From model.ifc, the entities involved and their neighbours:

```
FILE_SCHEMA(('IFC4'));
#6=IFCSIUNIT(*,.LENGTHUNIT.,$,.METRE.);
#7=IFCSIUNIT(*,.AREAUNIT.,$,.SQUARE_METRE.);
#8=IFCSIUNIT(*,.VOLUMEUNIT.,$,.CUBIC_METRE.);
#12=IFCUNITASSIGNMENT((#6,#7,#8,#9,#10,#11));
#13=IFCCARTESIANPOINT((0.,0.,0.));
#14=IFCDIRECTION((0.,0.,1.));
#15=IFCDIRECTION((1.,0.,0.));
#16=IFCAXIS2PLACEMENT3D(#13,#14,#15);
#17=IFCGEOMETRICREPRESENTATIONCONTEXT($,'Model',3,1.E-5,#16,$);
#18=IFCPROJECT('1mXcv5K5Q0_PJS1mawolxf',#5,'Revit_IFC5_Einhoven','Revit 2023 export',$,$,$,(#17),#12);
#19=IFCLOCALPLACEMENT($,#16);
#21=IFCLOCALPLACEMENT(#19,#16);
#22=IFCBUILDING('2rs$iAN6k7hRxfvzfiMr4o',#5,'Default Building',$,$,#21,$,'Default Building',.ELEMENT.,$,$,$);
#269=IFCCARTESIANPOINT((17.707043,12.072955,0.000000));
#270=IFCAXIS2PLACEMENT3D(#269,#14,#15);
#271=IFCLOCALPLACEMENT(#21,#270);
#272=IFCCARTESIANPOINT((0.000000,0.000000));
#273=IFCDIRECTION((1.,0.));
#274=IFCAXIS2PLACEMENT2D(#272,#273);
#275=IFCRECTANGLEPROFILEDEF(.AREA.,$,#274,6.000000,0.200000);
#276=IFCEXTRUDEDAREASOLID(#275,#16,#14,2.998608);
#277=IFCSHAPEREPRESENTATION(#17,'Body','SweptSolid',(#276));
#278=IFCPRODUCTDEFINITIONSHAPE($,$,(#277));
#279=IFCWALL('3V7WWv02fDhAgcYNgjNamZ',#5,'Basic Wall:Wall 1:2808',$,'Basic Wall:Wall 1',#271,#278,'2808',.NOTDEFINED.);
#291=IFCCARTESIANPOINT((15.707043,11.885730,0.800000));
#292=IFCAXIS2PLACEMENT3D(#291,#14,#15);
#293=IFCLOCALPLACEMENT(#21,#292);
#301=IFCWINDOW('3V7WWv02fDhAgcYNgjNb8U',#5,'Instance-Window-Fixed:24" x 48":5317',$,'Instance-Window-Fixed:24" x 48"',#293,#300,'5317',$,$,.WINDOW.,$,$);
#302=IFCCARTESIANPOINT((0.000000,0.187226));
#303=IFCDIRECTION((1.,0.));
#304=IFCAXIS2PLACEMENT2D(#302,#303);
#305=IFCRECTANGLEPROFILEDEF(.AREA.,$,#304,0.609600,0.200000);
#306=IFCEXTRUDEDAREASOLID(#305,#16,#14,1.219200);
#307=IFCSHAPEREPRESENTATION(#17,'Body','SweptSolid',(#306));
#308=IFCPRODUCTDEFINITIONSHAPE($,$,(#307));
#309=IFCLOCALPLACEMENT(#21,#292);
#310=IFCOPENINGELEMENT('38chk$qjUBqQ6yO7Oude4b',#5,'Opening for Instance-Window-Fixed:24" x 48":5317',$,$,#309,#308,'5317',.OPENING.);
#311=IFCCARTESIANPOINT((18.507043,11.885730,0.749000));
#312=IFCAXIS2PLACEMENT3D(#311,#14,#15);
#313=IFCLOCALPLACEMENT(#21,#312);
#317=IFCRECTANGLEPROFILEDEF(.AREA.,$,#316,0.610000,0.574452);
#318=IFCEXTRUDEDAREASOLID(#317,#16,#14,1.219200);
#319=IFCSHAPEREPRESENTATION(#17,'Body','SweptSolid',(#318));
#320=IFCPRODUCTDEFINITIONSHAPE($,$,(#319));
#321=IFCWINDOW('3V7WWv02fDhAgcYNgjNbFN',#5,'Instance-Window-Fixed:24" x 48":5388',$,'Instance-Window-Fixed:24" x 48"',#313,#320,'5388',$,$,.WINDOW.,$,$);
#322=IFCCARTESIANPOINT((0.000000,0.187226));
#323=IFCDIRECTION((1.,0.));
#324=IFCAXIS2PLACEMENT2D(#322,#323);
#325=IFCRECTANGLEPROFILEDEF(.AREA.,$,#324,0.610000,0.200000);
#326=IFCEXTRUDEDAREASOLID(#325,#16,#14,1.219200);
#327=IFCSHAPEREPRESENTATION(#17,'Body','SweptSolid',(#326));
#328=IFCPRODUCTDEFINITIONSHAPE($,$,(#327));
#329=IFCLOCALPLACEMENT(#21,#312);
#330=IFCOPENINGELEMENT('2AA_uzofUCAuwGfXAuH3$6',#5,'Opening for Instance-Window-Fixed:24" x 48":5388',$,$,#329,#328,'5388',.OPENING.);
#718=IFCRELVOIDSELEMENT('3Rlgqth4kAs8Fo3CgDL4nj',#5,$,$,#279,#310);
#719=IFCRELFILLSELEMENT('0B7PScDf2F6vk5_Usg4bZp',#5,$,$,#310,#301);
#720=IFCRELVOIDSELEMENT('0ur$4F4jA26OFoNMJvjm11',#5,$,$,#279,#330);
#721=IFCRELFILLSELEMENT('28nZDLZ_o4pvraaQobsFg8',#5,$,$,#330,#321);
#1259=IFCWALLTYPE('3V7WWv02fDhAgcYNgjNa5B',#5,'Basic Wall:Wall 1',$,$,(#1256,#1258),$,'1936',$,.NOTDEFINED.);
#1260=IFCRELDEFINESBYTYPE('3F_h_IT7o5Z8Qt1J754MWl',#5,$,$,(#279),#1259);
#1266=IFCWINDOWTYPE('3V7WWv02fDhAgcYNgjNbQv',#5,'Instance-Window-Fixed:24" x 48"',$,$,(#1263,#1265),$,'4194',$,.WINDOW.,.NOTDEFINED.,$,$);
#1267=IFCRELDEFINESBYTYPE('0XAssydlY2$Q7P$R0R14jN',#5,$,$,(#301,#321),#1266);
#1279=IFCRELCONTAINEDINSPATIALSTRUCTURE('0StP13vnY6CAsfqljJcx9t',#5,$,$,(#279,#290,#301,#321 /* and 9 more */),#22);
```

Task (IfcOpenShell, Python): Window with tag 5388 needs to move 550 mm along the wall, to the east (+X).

```python
import ifcopenshell
import ifcopenshell.api.geometry
import ifcopenshell.util.placement
import ifcopenshell.util.unit

model = ifcopenshell.open("model.ifc")
unit_scale = ifcopenshell.util.unit.calculate_unit_scale(model)

window = model.by_guid("3V7WWv02fDhAgcYNgjNbFN")
opening = window.FillsVoids[0].RelatingOpeningElement
wall = opening.VoidsElements[0].RelatingBuildingElement

wall_matrix = ifcopenshell.util.placement.get_local_placement(wall.ObjectPlacement)
shift = wall_matrix[:3, 0] * 0.55 / unit_scale
before = ifcopenshell.util.placement.get_local_placement(window.ObjectPlacement)[:3, 3].copy()

# The window is not placed relative to its opening, so move both.
for product in (opening, window):
    matrix = ifcopenshell.util.placement.get_local_placement(product.ObjectPlacement)
    matrix[:3, 3] += shift
    ifcopenshell.api.geometry.edit_object_placement(model, product=product, matrix=matrix, is_si=False)

after = ifcopenshell.util.placement.get_local_placement(window.ObjectPlacement)[:3, 3]
print("window moved by", (after - before).round(3) + 0.0)

model.write("model-out.ifc")
```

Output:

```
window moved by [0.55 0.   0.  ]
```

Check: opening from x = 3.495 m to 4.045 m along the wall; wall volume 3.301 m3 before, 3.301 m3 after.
